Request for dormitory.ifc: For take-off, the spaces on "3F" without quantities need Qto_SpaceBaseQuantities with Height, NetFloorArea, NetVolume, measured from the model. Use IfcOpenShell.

First a look at what the model holds.

```python
import ifcopenshell
import ifcopenshell.util.element
import ifcopenshell.util.unit

model = ifcopenshell.open("dormitory.ifc")
print(model.schema)
for unit_type in ("LENGTHUNIT", "AREAUNIT", "VOLUMEUNIT"):
    print(unit_type, ifcopenshell.util.unit.calculate_unit_scale(model, unit_type))
storey = next(s for s in model.by_type("IfcBuildingStorey") if s.Name == "3F")
spaces = [e for e in ifcopenshell.util.element.get_decomposition(storey) if e.is_a("IfcSpace")]
for e in sorted(spaces, key=lambda e: e.id()):
    print(e.id(), e.is_a(), e.Name, list(ifcopenshell.util.element.get_psets(e, qtos_only=True)), sep=" | ")
```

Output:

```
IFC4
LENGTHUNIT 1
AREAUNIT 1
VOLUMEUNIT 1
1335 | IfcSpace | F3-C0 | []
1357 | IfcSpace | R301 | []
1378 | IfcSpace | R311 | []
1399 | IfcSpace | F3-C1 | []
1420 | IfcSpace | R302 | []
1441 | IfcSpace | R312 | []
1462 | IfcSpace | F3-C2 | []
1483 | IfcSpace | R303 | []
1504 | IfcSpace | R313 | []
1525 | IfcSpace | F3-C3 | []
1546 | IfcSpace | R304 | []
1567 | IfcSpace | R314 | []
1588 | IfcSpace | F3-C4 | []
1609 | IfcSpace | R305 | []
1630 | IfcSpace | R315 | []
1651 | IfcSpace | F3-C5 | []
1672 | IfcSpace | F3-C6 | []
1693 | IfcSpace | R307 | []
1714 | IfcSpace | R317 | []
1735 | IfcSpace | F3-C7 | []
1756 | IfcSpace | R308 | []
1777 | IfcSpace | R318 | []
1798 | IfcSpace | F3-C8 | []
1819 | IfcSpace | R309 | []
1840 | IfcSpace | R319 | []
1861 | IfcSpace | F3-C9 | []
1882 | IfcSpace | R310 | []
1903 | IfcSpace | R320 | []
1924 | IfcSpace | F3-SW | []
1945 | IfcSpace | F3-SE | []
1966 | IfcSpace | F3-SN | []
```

```python
import ifcopenshell
import ifcopenshell.api.pset
import ifcopenshell.geom
import ifcopenshell.util.element
import ifcopenshell.util.shape
import ifcopenshell.util.unit

model = ifcopenshell.open("dormitory.ifc")
unit_scale = ifcopenshell.util.unit.calculate_unit_scale(model)
area_scale = ifcopenshell.util.unit.calculate_unit_scale(model, "AREAUNIT")
volume_scale = ifcopenshell.util.unit.calculate_unit_scale(model, "VOLUMEUNIT")
settings = ifcopenshell.geom.settings()

storey = next(s for s in model.by_type("IfcBuildingStorey") if s.Name == "3F")
spaces = [e for e in ifcopenshell.util.element.get_decomposition(storey) if e.is_a("IfcSpace")]

for e in sorted(spaces, key=lambda e: e.id()):
    if ifcopenshell.util.element.get_psets(e, qtos_only=True, should_inherit=False):
        continue
    # Geometry comes back in metres, in the element's own axes.
    shape = ifcopenshell.geom.create_shape(settings, e)
    values = {
        "Height": ifcopenshell.util.shape.get_z(shape.geometry) / unit_scale,
        "NetFloorArea": ifcopenshell.util.shape.get_footprint_area(shape.geometry) / area_scale,
        "NetVolume": ifcopenshell.util.shape.get_volume(shape.geometry) / volume_scale,
    }
    qto = ifcopenshell.api.pset.add_qto(model, product=e, name="Qto_SpaceBaseQuantities")
    ifcopenshell.api.pset.edit_qto(model, qto=qto, properties=values)
    print(e.id(), {k: round(v, 3) for k, v in values.items()})

model.write("dormitory_edited.ifc")
```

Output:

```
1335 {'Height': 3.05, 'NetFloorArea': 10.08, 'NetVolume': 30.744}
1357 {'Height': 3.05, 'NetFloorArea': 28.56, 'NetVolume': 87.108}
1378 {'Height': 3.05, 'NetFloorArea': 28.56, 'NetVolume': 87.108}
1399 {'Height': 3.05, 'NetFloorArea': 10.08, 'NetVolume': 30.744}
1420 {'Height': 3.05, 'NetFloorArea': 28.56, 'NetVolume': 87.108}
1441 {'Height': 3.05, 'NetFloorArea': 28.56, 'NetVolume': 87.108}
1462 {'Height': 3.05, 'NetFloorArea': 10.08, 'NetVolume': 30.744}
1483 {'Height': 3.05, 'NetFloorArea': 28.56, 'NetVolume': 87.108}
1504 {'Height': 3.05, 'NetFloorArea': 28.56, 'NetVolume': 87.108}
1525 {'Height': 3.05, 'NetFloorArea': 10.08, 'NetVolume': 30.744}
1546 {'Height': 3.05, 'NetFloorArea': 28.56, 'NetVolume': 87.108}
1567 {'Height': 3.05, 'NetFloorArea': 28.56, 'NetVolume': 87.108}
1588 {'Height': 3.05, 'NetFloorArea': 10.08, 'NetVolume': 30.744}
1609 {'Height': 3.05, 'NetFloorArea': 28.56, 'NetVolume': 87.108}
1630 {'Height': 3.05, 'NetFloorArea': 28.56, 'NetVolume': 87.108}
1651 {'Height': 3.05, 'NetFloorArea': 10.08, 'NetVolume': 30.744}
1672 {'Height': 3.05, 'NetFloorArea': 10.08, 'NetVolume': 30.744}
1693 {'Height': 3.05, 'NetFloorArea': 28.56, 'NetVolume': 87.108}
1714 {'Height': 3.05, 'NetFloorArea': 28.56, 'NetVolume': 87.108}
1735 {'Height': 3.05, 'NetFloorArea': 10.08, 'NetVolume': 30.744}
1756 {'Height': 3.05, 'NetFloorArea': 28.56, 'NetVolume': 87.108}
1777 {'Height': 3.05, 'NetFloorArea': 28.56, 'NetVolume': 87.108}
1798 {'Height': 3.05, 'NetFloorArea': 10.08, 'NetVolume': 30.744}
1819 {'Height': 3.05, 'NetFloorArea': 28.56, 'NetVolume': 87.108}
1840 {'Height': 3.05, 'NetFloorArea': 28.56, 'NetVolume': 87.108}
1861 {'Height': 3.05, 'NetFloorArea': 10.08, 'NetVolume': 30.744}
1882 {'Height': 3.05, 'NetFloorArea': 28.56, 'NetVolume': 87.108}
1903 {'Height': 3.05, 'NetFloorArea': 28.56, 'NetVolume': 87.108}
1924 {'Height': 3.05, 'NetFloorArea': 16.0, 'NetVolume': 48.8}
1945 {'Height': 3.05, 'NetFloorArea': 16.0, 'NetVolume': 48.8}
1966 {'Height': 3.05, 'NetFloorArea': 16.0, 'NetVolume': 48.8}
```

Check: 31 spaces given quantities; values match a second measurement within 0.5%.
